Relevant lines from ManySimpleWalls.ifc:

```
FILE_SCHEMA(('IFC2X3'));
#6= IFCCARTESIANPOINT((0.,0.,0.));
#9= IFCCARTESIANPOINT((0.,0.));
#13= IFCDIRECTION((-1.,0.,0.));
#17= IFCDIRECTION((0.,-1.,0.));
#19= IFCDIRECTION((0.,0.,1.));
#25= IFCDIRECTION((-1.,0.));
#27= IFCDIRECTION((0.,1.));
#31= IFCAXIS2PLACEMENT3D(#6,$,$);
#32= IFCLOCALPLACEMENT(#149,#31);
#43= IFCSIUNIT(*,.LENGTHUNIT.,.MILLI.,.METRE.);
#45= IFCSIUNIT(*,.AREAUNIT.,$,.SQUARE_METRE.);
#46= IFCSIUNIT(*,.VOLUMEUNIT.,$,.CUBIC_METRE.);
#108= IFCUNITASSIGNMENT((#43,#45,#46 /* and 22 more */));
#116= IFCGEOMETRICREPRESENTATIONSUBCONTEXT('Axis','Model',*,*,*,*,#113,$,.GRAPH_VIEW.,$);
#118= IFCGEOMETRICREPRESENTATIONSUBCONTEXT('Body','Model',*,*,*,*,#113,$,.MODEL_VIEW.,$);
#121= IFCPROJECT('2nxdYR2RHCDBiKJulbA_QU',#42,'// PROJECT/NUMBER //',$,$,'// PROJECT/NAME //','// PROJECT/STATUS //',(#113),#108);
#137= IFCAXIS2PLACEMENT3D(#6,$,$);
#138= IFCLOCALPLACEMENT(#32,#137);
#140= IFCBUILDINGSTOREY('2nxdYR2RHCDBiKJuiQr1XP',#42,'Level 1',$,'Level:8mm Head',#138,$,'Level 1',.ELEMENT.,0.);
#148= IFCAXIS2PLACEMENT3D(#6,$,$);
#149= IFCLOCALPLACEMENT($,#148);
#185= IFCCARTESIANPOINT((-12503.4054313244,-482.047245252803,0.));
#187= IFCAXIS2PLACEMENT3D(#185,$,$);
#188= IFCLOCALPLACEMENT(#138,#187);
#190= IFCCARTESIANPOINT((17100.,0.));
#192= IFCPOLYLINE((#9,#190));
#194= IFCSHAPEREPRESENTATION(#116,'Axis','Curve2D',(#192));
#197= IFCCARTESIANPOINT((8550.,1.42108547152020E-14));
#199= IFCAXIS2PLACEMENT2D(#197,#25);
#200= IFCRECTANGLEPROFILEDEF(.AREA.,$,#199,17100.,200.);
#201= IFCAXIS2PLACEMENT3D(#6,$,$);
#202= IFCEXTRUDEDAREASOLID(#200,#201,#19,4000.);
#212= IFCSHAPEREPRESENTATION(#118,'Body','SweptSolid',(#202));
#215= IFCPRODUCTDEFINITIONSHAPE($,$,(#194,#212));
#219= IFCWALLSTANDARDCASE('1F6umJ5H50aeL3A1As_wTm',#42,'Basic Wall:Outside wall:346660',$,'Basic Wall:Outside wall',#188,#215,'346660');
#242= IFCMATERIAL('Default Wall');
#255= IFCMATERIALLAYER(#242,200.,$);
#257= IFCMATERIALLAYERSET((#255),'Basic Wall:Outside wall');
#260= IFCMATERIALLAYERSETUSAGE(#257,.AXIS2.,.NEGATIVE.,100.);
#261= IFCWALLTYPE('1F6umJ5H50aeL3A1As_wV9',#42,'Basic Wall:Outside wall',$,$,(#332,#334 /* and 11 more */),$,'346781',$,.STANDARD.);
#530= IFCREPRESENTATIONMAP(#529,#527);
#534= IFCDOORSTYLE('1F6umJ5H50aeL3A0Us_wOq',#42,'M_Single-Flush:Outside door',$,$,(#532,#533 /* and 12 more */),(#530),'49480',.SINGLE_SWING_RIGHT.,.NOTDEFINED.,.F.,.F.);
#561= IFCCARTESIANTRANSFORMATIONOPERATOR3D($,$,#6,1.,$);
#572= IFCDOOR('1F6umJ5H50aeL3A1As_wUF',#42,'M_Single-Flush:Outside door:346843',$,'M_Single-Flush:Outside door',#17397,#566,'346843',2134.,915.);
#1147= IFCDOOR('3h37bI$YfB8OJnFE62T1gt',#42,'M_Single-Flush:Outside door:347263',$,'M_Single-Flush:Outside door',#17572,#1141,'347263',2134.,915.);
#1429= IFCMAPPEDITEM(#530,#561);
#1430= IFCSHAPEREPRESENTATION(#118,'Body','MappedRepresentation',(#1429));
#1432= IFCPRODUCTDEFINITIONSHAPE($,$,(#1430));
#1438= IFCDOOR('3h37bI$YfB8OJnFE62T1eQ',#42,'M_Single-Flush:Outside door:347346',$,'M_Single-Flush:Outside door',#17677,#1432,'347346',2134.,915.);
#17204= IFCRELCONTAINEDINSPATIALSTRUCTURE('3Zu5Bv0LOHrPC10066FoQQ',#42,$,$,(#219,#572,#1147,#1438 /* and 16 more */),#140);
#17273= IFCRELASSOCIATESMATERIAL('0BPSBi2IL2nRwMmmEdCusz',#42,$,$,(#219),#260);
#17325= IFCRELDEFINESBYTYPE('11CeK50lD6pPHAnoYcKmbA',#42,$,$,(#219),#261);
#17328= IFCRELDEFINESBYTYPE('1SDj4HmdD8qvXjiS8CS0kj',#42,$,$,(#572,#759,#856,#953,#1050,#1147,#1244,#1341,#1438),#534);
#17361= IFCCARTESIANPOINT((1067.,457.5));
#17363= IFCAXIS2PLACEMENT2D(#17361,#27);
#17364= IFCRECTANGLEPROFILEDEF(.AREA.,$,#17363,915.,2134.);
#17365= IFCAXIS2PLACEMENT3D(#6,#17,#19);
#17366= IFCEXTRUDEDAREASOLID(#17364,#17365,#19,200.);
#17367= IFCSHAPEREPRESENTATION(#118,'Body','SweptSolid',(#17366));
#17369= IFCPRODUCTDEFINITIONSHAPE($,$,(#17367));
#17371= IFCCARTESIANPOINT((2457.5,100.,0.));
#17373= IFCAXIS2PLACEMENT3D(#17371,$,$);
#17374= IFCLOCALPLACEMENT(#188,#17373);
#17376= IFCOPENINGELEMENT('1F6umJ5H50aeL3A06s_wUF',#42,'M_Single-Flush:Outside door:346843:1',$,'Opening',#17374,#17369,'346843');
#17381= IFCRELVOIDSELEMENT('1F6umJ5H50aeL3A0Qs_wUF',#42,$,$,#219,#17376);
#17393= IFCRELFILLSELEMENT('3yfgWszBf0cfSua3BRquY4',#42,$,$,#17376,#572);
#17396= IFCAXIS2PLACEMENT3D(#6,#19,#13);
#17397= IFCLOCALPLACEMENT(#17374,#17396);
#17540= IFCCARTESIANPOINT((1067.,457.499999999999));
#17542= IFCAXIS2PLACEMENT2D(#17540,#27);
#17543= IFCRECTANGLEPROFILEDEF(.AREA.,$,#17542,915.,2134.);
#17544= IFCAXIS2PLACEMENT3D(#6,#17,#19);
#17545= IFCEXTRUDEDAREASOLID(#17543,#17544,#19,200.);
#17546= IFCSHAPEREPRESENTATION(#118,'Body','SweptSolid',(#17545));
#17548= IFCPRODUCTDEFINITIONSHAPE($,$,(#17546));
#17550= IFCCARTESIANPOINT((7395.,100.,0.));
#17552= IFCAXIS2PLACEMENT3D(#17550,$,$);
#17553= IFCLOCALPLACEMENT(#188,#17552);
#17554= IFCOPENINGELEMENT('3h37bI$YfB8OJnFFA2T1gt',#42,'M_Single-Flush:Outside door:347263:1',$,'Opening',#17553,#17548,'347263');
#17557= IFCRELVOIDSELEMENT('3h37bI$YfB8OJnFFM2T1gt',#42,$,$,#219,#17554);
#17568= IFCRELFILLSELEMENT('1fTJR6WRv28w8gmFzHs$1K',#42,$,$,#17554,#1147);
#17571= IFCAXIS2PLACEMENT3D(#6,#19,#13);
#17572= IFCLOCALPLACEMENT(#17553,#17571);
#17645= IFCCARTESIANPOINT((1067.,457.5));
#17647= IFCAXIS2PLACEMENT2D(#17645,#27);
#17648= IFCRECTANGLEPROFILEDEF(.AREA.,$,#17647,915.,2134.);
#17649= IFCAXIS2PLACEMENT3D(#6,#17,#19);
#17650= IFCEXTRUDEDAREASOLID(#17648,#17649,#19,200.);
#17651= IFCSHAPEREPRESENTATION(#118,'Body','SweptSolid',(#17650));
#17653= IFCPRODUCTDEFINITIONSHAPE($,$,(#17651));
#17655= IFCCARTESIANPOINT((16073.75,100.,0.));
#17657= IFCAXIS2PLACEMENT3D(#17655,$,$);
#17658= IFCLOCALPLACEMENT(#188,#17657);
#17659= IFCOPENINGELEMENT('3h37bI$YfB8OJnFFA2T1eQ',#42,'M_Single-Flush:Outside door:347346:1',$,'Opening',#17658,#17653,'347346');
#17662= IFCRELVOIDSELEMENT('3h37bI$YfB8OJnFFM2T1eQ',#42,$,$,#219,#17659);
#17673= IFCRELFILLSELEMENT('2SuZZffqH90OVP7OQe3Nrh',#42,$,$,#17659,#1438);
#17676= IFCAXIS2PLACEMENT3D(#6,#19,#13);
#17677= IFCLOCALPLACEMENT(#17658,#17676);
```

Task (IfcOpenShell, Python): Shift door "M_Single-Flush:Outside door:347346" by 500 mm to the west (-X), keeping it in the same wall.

```python
import ifcopenshell
import ifcopenshell.api.geometry
import ifcopenshell.util.placement
import ifcopenshell.util.unit

model = ifcopenshell.open("ManySimpleWalls.ifc")
unit_scale = ifcopenshell.util.unit.calculate_unit_scale(model)

door = model.by_id(1438)
opening = door.FillsVoids[0].RelatingOpeningElement
wall = opening.VoidsElements[0].RelatingBuildingElement

wall_matrix = ifcopenshell.util.placement.get_local_placement(wall.ObjectPlacement)
shift = wall_matrix[:3, 0] * -0.5 / unit_scale
before = ifcopenshell.util.placement.get_local_placement(door.ObjectPlacement)[:3, 3].copy()

# The door is placed relative to its opening, so it follows when the opening moves.
matrix = ifcopenshell.util.placement.get_local_placement(opening.ObjectPlacement)
matrix[:3, 3] += shift
ifcopenshell.api.geometry.edit_object_placement(
    model, product=opening, matrix=matrix, is_si=False, should_transform_children=True
)

after = ifcopenshell.util.placement.get_local_placement(door.ObjectPlacement)[:3, 3]
print("door moved by", (after - before).round(3) + 0.0)

model.write("ManySimpleWalls_updated.ifc")
```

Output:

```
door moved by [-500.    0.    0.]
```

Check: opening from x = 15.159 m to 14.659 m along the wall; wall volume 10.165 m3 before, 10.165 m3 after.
